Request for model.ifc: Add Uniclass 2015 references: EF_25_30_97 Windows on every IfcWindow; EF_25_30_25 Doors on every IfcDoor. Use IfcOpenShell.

First a look at what the model holds.

```python
import ifcopenshell

model = ifcopenshell.open("model.ifc")
print(model.schema)
print("classifications:", [c.Name for c in model.by_type("IfcClassification")])
for ifc_class in ("IfcDoor", "IfcRoof", "IfcStair", "IfcWall", "IfcWindow"):
    print(ifc_class, len(model.by_type(ifc_class)))
```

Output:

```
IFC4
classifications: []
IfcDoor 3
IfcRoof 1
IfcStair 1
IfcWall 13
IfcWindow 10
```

```python
import ifcopenshell
import ifcopenshell.api.classification

model = ifcopenshell.open("model.ifc")

system = ifcopenshell.api.classification.add_classification(model, classification="Uniclass 2015")

codes = {
    "IfcWindow": ("EF_25_30_97", "Windows"),
    "IfcDoor": ("EF_25_30_25", "Doors"),
}
for ifc_class, (code, name) in codes.items():
    products = model.by_type(ifc_class)
    ifcopenshell.api.classification.add_reference(
        model, products=products, classification=system, identification=code, name=name
    )
    print(code, len(products))

model.write("model_rev.ifc")
```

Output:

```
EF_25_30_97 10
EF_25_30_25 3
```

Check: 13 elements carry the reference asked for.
